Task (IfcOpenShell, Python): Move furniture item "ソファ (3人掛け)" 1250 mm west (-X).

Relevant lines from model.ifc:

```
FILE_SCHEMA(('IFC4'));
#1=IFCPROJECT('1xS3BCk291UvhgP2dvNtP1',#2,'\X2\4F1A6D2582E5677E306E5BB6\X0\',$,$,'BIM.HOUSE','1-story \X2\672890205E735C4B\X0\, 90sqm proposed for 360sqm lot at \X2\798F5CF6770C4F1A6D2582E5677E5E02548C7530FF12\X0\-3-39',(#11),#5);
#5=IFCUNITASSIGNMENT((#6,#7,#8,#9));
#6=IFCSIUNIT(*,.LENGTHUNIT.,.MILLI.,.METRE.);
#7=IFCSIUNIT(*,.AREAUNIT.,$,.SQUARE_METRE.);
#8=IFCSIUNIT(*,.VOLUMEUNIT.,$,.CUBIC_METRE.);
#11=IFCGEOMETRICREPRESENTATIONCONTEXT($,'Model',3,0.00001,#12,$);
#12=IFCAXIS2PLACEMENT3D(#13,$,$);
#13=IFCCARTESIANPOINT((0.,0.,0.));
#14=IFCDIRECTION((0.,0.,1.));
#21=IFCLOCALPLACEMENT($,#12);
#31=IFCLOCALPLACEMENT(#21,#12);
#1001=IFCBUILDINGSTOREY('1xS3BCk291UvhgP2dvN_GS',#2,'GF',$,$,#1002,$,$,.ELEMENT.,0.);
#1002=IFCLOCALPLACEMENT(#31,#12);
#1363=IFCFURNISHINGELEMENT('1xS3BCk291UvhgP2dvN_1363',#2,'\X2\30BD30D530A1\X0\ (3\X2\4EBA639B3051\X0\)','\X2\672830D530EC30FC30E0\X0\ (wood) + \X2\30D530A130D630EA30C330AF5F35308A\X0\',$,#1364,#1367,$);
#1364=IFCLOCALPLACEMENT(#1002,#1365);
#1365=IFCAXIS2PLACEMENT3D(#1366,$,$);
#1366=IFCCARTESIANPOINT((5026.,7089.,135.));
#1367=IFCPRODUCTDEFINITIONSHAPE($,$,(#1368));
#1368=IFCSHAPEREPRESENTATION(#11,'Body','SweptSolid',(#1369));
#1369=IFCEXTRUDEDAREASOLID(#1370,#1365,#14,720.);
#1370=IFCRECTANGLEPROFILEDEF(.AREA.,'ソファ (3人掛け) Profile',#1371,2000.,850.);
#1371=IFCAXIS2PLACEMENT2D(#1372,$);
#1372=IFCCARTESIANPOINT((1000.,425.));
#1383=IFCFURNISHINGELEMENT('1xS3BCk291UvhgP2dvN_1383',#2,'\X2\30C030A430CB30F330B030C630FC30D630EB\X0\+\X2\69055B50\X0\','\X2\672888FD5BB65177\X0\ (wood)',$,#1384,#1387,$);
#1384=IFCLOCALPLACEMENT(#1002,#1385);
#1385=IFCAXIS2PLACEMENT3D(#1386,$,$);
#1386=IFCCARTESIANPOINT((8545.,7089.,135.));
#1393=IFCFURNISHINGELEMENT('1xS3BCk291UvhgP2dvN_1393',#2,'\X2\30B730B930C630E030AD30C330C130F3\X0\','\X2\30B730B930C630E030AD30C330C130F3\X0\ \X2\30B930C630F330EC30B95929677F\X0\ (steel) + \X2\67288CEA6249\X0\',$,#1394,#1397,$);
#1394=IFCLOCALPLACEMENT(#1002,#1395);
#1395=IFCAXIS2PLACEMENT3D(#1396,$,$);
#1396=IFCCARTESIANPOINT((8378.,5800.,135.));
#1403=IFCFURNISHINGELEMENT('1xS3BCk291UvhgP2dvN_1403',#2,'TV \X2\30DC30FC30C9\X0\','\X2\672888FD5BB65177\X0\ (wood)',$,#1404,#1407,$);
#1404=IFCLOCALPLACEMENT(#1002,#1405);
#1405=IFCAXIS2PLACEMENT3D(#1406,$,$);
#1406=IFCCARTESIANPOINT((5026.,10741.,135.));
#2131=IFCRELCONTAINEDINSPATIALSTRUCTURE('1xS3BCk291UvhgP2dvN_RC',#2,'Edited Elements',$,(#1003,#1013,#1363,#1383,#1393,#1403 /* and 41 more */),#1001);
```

```python
import ifcopenshell
import ifcopenshell.api.geometry
import ifcopenshell.util.placement
import ifcopenshell.util.unit

model = ifcopenshell.open("model.ifc")
unit_scale = ifcopenshell.util.unit.calculate_unit_scale(model)

item = model.by_id(1363)
matrix = ifcopenshell.util.placement.get_local_placement(item.ObjectPlacement)
matrix[0, 3] -= 1.25 / unit_scale
ifcopenshell.api.geometry.edit_object_placement(model, product=item, matrix=matrix, is_si=False)

print(ifcopenshell.util.placement.get_local_placement(item.ObjectPlacement).round(3) + 0.0)

model.write("model-out.ifc")
```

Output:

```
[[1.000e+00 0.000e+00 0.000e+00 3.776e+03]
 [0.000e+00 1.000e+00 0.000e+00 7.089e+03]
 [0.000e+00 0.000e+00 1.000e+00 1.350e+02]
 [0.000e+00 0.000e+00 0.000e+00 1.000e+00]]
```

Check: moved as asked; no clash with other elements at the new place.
